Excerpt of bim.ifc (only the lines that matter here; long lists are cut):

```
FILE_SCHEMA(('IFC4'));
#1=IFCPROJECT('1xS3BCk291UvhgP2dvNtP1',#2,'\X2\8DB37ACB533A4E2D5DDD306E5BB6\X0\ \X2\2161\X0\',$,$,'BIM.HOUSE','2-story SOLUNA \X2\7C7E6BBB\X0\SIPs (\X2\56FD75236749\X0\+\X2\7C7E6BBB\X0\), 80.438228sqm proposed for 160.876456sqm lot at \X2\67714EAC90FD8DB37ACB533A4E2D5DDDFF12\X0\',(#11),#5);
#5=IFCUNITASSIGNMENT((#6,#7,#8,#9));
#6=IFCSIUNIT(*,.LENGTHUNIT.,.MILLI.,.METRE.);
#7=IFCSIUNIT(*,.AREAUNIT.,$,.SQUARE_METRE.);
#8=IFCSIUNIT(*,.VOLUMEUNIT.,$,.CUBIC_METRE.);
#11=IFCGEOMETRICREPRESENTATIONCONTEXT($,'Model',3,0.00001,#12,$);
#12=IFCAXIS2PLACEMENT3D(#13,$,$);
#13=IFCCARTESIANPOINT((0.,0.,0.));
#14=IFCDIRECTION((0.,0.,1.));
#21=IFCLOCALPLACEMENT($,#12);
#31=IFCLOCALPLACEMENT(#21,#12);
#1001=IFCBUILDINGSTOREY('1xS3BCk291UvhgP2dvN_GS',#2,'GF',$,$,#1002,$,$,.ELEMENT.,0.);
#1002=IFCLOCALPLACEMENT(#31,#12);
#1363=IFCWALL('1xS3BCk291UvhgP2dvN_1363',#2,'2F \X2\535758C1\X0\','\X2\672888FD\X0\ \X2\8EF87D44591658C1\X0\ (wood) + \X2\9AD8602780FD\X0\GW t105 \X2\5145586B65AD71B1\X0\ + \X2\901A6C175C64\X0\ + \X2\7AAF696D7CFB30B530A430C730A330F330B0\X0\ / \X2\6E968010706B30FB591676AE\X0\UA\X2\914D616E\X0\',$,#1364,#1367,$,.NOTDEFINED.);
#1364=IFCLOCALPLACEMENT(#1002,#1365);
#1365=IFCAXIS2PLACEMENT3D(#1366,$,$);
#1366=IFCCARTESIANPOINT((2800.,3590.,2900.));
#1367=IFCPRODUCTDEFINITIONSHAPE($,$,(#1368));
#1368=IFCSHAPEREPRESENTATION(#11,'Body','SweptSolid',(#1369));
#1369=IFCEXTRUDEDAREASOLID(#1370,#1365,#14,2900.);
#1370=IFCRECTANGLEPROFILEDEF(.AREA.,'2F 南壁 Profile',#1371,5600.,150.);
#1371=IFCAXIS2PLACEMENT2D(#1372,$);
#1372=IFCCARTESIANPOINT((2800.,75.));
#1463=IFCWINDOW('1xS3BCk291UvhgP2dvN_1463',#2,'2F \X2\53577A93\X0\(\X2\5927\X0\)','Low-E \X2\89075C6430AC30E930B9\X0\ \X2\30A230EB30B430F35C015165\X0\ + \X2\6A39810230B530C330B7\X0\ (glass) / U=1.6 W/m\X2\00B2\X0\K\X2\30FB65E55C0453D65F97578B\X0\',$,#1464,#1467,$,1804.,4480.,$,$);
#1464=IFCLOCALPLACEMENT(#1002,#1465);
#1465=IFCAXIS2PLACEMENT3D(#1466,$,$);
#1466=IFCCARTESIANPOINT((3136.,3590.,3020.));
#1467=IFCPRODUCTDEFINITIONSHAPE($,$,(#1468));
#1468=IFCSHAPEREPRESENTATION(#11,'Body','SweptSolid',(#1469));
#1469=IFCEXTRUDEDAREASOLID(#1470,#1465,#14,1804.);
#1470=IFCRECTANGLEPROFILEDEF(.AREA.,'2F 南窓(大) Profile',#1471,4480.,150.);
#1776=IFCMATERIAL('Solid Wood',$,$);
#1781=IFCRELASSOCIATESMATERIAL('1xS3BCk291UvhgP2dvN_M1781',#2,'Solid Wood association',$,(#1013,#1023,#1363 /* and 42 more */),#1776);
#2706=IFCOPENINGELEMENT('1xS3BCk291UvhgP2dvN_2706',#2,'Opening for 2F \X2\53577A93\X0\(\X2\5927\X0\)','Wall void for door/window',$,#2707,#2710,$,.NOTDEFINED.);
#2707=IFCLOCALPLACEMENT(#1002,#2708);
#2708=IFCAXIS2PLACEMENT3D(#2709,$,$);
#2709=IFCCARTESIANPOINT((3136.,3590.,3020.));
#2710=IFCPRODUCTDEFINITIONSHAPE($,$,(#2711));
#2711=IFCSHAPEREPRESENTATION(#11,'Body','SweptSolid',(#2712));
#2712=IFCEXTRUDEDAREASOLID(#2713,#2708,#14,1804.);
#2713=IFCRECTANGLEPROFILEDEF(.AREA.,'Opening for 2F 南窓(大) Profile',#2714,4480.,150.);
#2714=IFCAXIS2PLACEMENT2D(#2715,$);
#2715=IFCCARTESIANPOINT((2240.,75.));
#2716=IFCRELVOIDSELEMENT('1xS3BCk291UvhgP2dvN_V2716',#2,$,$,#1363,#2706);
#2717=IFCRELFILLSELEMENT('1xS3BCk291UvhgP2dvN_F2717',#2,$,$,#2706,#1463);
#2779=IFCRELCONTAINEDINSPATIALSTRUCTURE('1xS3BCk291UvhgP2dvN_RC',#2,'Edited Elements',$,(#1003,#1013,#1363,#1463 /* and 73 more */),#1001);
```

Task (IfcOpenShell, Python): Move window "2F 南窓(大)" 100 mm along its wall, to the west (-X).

```python
import ifcopenshell
import ifcopenshell.api.geometry
import ifcopenshell.util.placement
import ifcopenshell.util.unit

model = ifcopenshell.open("bim.ifc")
unit_scale = ifcopenshell.util.unit.calculate_unit_scale(model)

window = model.by_guid("1xS3BCk291UvhgP2dvN_1463")
opening = window.FillsVoids[0].RelatingOpeningElement
wall = opening.VoidsElements[0].RelatingBuildingElement

wall_matrix = ifcopenshell.util.placement.get_local_placement(wall.ObjectPlacement)
shift = wall_matrix[:3, 0] * -0.1 / unit_scale
before = ifcopenshell.util.placement.get_local_placement(window.ObjectPlacement)[:3, 3].copy()

# The window is not placed relative to its opening, so move both.
for product in (opening, window):
    matrix = ifcopenshell.util.placement.get_local_placement(product.ObjectPlacement)
    matrix[:3, 3] += shift
    ifcopenshell.api.geometry.edit_object_placement(model, product=product, matrix=matrix, is_si=False)

after = ifcopenshell.util.placement.get_local_placement(window.ObjectPlacement)[:3, 3]
print("window moved by", (after - before).round(3) + 0.0)

model.write("bim-out.ifc")
```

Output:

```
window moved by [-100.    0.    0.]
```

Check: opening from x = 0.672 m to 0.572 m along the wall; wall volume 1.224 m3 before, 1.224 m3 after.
